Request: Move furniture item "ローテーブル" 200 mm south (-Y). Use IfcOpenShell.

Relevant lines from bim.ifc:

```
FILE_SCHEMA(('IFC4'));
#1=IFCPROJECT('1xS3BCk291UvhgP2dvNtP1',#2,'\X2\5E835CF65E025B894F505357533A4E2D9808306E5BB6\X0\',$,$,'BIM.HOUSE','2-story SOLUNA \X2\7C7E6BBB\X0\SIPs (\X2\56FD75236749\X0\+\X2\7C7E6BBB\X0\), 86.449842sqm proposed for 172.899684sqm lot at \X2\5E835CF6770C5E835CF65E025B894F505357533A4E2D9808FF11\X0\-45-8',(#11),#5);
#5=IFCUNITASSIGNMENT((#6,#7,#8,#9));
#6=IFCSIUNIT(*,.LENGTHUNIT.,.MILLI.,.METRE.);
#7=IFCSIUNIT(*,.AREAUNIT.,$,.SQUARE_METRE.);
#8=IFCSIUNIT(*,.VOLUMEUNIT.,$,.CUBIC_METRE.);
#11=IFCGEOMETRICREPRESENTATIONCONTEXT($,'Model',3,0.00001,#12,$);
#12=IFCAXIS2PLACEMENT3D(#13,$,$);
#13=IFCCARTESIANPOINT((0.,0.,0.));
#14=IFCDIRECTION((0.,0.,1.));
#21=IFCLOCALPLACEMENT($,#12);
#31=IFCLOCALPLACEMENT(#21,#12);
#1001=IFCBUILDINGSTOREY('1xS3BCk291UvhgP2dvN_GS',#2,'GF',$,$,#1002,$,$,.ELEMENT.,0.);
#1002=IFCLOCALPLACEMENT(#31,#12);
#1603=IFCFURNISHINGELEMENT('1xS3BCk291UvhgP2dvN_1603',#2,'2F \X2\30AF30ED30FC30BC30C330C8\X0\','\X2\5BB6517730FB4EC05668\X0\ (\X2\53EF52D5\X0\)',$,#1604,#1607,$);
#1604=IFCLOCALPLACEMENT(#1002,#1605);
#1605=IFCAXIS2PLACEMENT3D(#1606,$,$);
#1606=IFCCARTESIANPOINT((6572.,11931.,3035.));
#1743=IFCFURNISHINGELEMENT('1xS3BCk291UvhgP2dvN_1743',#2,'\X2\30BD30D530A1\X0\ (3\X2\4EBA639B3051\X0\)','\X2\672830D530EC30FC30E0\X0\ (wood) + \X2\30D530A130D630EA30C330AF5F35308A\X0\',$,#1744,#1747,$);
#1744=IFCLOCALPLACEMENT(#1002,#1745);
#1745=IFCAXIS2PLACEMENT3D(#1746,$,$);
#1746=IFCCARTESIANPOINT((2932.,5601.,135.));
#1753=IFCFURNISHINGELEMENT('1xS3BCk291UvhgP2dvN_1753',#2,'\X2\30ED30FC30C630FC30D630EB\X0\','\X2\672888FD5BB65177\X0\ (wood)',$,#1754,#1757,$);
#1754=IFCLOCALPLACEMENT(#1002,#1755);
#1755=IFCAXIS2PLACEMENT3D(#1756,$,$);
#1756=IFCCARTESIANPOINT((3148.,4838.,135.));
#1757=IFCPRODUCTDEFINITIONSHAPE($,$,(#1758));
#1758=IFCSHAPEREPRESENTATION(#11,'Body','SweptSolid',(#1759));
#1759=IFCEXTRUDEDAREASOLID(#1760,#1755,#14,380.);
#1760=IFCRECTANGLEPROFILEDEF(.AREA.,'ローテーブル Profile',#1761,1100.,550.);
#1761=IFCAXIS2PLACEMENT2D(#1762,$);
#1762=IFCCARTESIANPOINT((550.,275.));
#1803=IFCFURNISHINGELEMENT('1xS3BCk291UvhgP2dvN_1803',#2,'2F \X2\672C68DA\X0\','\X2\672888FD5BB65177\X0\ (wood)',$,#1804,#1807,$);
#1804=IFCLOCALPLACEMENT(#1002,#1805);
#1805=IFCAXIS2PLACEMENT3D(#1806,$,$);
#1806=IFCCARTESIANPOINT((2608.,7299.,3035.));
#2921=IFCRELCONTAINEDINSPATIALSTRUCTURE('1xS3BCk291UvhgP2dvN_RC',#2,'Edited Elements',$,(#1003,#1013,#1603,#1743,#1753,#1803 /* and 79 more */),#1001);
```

```python
import ifcopenshell
import ifcopenshell.api.geometry
import ifcopenshell.util.placement
import ifcopenshell.util.unit

model = ifcopenshell.open("bim.ifc")
unit_scale = ifcopenshell.util.unit.calculate_unit_scale(model)

item = model.by_guid("1xS3BCk291UvhgP2dvN_1753")
matrix = ifcopenshell.util.placement.get_local_placement(item.ObjectPlacement)
matrix[1, 3] -= 0.2 / unit_scale
ifcopenshell.api.geometry.edit_object_placement(model, product=item, matrix=matrix, is_si=False)

print(ifcopenshell.util.placement.get_local_placement(item.ObjectPlacement).round(3) + 0.0)

model.write("bim_v2.ifc")
```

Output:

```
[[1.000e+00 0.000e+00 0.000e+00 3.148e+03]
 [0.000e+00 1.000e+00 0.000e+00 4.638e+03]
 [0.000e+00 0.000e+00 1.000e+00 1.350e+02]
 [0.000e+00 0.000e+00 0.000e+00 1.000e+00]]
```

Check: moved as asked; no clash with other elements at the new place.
